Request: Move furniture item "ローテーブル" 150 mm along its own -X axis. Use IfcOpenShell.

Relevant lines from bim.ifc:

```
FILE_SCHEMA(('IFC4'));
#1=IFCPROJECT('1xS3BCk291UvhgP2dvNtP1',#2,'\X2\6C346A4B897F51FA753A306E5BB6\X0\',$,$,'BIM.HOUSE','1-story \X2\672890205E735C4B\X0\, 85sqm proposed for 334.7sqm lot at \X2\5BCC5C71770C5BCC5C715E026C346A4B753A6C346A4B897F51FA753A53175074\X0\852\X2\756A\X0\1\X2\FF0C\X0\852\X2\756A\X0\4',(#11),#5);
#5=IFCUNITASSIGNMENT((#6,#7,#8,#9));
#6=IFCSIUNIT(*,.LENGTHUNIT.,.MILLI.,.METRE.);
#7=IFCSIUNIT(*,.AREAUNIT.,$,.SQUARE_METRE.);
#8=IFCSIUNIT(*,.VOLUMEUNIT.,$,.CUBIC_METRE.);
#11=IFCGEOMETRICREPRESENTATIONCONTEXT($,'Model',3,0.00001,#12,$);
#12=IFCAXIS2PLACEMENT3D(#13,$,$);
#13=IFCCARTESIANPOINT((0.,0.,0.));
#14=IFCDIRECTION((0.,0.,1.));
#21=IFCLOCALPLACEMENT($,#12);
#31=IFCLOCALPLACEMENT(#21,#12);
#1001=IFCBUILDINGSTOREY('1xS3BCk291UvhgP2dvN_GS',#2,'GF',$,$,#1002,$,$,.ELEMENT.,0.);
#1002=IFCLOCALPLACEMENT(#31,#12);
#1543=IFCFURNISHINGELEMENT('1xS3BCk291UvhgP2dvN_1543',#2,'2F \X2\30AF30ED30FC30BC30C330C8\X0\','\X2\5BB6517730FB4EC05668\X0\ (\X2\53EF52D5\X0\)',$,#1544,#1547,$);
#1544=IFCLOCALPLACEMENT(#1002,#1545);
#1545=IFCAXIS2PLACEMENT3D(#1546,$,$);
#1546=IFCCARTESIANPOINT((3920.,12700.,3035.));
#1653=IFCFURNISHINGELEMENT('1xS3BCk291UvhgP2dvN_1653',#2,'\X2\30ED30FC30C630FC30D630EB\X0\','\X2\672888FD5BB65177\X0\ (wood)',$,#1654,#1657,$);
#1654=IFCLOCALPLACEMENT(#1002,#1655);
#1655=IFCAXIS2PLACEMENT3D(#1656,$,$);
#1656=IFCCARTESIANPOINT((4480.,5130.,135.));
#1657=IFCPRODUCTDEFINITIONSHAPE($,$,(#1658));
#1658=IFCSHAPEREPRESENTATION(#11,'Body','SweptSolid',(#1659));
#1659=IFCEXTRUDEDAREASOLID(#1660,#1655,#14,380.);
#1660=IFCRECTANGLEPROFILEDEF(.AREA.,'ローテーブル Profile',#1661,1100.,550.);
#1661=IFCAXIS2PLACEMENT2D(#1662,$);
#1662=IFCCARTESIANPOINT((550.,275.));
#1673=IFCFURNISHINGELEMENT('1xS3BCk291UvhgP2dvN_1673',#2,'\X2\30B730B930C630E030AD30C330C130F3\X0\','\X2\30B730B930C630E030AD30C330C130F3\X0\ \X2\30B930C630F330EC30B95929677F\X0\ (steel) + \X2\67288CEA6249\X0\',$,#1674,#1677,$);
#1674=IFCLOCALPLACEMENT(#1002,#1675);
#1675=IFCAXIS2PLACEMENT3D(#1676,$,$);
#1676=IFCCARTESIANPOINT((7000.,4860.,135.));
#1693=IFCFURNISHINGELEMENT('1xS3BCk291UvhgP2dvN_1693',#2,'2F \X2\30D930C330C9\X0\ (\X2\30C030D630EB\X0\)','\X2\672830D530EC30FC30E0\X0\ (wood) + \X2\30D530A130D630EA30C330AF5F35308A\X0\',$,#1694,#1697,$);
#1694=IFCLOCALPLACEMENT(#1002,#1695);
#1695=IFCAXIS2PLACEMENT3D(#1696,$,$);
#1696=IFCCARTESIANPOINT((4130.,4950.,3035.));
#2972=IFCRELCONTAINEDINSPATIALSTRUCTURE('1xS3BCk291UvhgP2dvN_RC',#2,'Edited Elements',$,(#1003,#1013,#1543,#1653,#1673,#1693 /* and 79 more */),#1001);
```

```python
import ifcopenshell
import ifcopenshell.api.geometry
import ifcopenshell.util.placement
import ifcopenshell.util.unit

model = ifcopenshell.open("bim.ifc")
unit_scale = ifcopenshell.util.unit.calculate_unit_scale(model)

item = model.by_guid("1xS3BCk291UvhgP2dvN_1653")
matrix = ifcopenshell.util.placement.get_local_placement(item.ObjectPlacement)
matrix[:3, 3] -= matrix[:3, 0] * 0.15 / unit_scale
ifcopenshell.api.geometry.edit_object_placement(model, product=item, matrix=matrix, is_si=False)

print(ifcopenshell.util.placement.get_local_placement(item.ObjectPlacement).round(3) + 0.0)

model.write("bim-out.ifc")
```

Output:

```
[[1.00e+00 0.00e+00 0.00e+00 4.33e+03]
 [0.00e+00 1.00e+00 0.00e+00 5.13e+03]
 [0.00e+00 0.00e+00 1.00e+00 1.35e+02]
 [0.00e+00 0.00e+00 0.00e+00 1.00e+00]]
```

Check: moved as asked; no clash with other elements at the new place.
